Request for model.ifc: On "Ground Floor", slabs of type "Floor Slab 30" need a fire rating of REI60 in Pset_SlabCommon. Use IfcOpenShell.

First a look at what the model holds.

```python
import ifcopenshell
import ifcopenshell.util.element

model = ifcopenshell.open("model.ifc")
print(model.schema)
storey = next(s for s in model.by_type("IfcBuildingStorey") if s.Name == "Ground Floor")
slabs = [e for e in ifcopenshell.util.element.get_decomposition(storey) if e.is_a("IfcSlab")]
seen = {}
for e in slabs:
    element_type = ifcopenshell.util.element.get_type(e)
    key = (element_type.Name if element_type != e and element_type else None, ifcopenshell.util.element.get_pset(e, "Pset_SlabCommon", "FireRating"))
    seen[key] = seen.get(key, 0) + 1
for (name, value), count in sorted(seen.items(), key=str):
    print(count, "x", name, "|", value)
```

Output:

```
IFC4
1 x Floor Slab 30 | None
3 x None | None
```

```python
import ifcopenshell
import ifcopenshell.api.pset
import ifcopenshell.util.element

model = ifcopenshell.open("model.ifc")

storey = next(s for s in model.by_type("IfcBuildingStorey") if s.Name == "Ground Floor")
slabs = [e for e in ifcopenshell.util.element.get_decomposition(storey) if e.is_a("IfcSlab")]

count = 0
for e in slabs:
    element_type = ifcopenshell.util.element.get_type(e)
    if element_type in (None, e) or element_type.Name != "Floor Slab 30":
        continue
    # add_pset returns the element's existing set when there is one.
    pset = ifcopenshell.api.pset.add_pset(model, product=e, name="Pset_SlabCommon")
    ifcopenshell.api.pset.edit_pset(model, pset=pset, properties={"FireRating": "REI60"})
    count += 1

print(count, "slabs updated")

model.write("model_edited.ifc")
```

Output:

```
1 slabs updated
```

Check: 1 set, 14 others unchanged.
